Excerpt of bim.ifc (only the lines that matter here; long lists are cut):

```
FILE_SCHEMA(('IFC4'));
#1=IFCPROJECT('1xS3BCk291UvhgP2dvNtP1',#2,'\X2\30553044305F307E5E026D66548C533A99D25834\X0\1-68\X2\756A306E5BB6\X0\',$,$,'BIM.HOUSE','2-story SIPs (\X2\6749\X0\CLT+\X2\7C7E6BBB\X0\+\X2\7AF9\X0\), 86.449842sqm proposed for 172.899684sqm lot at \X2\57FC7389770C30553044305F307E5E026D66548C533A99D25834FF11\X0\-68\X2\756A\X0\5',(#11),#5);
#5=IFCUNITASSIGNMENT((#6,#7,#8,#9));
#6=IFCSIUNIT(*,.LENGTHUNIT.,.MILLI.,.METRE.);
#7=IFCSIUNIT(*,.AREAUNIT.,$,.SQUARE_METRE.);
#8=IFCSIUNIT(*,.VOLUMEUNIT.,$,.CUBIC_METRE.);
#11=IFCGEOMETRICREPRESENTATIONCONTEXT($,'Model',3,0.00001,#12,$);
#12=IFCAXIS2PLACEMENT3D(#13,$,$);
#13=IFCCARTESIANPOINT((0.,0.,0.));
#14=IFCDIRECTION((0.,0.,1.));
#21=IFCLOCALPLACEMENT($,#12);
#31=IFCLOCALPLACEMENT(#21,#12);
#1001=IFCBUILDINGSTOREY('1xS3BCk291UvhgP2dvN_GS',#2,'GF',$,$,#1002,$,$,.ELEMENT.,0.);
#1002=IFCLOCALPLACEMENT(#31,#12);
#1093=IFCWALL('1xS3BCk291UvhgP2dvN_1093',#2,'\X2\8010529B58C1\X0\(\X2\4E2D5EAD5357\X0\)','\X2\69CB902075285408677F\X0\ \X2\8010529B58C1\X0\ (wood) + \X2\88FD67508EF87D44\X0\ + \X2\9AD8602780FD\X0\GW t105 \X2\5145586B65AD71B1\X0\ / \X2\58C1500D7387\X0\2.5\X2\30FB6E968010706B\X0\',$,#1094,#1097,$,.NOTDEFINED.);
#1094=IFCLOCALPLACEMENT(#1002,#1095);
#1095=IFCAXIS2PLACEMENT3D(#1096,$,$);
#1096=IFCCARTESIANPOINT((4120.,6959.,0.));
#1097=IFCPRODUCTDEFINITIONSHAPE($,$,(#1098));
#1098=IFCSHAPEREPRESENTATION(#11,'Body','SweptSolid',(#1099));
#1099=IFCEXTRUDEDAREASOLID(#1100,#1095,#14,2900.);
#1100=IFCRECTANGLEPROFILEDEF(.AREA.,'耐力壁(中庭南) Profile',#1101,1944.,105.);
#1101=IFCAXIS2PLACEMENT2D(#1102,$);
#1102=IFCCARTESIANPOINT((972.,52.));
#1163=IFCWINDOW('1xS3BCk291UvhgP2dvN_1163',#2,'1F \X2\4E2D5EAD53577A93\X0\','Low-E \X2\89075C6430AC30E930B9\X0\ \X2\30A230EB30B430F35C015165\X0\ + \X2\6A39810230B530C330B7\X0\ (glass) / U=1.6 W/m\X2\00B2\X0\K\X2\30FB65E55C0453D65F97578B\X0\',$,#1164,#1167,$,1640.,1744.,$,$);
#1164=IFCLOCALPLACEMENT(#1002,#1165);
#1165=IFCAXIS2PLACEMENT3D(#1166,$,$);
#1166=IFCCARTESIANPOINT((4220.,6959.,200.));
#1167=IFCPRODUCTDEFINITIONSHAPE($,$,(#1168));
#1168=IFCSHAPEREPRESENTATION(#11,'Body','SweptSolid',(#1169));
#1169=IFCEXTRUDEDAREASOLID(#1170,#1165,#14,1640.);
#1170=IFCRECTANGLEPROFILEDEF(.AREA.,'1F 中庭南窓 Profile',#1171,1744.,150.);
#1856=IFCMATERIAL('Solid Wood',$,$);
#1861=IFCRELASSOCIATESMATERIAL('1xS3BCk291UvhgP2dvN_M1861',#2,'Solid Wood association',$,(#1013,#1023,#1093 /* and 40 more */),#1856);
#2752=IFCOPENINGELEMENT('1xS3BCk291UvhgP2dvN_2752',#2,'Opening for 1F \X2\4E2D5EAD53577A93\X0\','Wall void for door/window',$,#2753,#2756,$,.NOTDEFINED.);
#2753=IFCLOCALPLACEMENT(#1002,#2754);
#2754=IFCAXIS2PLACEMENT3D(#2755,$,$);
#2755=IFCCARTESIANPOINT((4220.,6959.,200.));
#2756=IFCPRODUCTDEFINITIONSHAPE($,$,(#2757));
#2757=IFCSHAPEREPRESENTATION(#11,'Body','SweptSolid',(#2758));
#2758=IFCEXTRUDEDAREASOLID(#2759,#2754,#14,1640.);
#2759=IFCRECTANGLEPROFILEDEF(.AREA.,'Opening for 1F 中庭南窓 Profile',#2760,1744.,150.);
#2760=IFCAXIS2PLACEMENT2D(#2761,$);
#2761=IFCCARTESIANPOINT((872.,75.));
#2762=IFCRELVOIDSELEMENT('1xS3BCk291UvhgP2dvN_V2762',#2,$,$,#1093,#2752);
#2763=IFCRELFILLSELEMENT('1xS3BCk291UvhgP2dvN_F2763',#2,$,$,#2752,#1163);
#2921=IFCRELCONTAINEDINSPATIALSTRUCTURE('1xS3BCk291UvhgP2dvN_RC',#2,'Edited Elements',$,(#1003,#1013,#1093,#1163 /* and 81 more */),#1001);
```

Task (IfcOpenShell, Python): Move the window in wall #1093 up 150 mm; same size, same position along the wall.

```python
import numpy as np
import ifcopenshell
import ifcopenshell.api.geometry
import ifcopenshell.util.placement
import ifcopenshell.util.unit

model = ifcopenshell.open("bim.ifc")
unit_scale = ifcopenshell.util.unit.calculate_unit_scale(model)

window = model.by_guid("1xS3BCk291UvhgP2dvN_1163")
opening = window.FillsVoids[0].RelatingOpeningElement
dz = 0.15 / unit_scale

shift = np.array([0.0, 0.0, dz])
# The window is not placed relative to its opening, so move both.
for product in (opening, window):
    matrix = ifcopenshell.util.placement.get_local_placement(product.ObjectPlacement)
    matrix[:3, 3] += shift
    ifcopenshell.api.geometry.edit_object_placement(model, product=product, matrix=matrix, is_si=False)

print(f"moved by {dz * unit_scale:+.3f} m")

model.write("bim_edited.ifc")
```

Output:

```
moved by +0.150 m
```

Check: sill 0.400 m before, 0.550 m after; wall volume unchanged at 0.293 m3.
